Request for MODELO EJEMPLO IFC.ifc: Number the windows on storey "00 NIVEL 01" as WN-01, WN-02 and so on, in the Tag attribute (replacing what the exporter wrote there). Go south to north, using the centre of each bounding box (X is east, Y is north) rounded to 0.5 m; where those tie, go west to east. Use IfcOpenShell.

First a look at what the model holds.

```python
import ifcopenshell
import ifcopenshell.util.element
import ifcopenshell.util.placement

model = ifcopenshell.open("MODELO EJEMPLO IFC.ifc")
print(model.schema)
storey = next(s for s in model.by_type("IfcBuildingStorey") if s.Name == "00 NIVEL 01")
windows = [e for e in ifcopenshell.util.element.get_decomposition(storey) if e.is_a("IfcWindow")]
for e in sorted(windows, key=lambda e: e.id()):
    origin = ifcopenshell.util.placement.get_local_placement(e.ObjectPlacement)[:3, 3]
    print(e.id(), e.Tag, e.Name, origin.round(2) + 0.0, sep=" | ")
```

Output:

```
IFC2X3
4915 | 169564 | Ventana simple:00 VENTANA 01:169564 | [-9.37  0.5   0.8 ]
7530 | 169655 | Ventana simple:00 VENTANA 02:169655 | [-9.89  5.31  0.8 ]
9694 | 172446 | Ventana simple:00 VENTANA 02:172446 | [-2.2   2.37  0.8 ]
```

```python
import ifcopenshell
import ifcopenshell.geom
import ifcopenshell.util.element
import ifcopenshell.util.shape

model = ifcopenshell.open("MODELO EJEMPLO IFC.ifc")
settings = ifcopenshell.geom.settings()
settings.set("use-world-coords", True)


def centre(element):
    shape = ifcopenshell.geom.create_shape(settings, element)
    return ifcopenshell.util.shape.get_bbox_centroid(shape.geometry)


storey = next(s for s in model.by_type("IfcBuildingStorey") if s.Name == "00 NIVEL 01")
windows = [e for e in ifcopenshell.util.element.get_decomposition(storey) if e.is_a("IfcWindow")]

# Insertion points can sit at a corner or the storey origin, so sort by the geometry (in metres).
centres = {e: centre(e) for e in windows}
windows.sort(key=lambda e: (round(centres[e][1] / 0.5), centres[e][0]))

for i, e in enumerate(windows, start=1):
    number = f"WN-{i:02d}"
    e.Tag = number
    print(e.id(), number)

model.write("MODELO EJEMPLO IFC_rev.ifc")
```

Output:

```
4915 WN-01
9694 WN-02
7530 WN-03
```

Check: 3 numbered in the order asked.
